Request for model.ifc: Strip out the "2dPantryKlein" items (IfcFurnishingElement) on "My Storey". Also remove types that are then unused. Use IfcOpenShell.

First a look at what the model holds.

```python
import ifcopenshell
import ifcopenshell.util.element

model = ifcopenshell.open("model.ifc")
print(model.schema)
storey = next(s for s in model.by_type("IfcBuildingStorey") if s.Name == "My Storey")
furniture = [e for e in ifcopenshell.util.element.get_decomposition(storey) if e.is_a("IfcFurnishingElement")]
seen = {}
for e in furniture:
    element_type = ifcopenshell.util.element.get_type(e)
    name = element_type.Name if element_type not in (None, e) else None
    seen[name] = seen.get(name, 0) + 1
for name, count in sorted(seen.items(), key=str):
    print(count, "x", name)
```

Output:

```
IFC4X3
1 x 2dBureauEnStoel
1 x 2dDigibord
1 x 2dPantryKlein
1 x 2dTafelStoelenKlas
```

```python
import ifcopenshell
import ifcopenshell.api.root
import ifcopenshell.util.element

model = ifcopenshell.open("model.ifc")

storey = next(s for s in model.by_type("IfcBuildingStorey") if s.Name == "My Storey")
furniture = [e for e in ifcopenshell.util.element.get_decomposition(storey) if e.is_a("IfcFurnishingElement")]
targets = [e for e in furniture if (t := ifcopenshell.util.element.get_type(e)) not in (None, e) and t.Name == "2dPantryKlein"]
types = {ifcopenshell.util.element.get_type(e) for e in targets} - {None, *targets}

for e in targets:
    ifcopenshell.api.root.remove_product(model, product=e)
print(len(targets), "removed")

unused = [t for t in types if not ifcopenshell.util.element.get_types(t)]
for t in unused:
    ifcopenshell.api.root.remove_product(model, product=t)
print(len(unused), "unused types removed")

model.write("model-out.ifc")
```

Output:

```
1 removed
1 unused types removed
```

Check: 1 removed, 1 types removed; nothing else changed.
